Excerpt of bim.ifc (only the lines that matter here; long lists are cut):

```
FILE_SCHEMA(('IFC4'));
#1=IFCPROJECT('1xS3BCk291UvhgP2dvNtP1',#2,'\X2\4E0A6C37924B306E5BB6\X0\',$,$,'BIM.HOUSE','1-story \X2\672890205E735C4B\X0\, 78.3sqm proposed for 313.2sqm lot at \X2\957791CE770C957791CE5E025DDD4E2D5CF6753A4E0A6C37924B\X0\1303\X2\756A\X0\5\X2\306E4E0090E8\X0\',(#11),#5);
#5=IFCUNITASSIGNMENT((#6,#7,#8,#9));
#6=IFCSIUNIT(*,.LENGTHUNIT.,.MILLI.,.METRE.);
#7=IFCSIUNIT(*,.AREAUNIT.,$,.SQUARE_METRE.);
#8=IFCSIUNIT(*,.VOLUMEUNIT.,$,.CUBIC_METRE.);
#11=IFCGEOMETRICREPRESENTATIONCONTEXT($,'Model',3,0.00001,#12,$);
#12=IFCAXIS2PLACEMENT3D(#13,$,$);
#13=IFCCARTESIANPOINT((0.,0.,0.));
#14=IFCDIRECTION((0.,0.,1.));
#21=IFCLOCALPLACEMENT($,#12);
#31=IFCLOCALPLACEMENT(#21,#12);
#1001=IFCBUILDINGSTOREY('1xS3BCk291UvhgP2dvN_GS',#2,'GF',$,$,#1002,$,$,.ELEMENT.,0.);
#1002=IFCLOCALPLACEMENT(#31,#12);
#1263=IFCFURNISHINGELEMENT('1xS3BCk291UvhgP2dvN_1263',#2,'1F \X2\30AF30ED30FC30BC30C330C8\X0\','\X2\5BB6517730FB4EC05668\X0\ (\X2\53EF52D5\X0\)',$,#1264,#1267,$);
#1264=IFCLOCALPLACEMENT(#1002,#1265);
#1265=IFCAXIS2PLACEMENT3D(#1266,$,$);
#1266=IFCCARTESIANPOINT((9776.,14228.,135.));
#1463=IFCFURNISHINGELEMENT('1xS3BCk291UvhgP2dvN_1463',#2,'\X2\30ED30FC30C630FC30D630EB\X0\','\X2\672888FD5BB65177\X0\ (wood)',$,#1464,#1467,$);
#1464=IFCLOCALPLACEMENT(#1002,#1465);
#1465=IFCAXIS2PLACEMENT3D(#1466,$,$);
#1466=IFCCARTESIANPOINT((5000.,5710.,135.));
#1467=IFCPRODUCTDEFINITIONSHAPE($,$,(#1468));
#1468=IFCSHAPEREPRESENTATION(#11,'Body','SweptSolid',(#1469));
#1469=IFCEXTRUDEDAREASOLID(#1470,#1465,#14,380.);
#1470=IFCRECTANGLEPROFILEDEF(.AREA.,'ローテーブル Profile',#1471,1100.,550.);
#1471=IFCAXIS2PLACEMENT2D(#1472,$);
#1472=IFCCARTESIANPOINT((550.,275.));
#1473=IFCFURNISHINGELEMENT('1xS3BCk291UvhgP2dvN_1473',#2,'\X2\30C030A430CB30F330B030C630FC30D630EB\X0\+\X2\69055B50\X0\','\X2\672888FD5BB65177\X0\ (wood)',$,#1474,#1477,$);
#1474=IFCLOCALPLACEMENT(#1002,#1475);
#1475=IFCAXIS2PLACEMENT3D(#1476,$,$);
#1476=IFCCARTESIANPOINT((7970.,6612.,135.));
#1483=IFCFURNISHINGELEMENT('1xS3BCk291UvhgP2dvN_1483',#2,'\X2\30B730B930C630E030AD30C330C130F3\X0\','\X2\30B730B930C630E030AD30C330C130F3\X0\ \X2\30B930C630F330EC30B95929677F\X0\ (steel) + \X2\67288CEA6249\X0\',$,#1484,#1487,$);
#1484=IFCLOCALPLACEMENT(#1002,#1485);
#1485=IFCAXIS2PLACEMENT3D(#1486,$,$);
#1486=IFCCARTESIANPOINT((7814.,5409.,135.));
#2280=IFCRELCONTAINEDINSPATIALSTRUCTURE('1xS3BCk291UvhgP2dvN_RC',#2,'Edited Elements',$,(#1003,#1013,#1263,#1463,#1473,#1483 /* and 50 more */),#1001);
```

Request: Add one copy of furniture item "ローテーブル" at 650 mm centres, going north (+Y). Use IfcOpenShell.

```python
import numpy as np
import ifcopenshell
import ifcopenshell.api.geometry
import ifcopenshell.api.root
import ifcopenshell.util.element
import ifcopenshell.util.placement

model = ifcopenshell.open("bim.ifc")


def reuse_history(source, copy):
    """copy_class also copies each property set's owner history, people and application; keep the originals."""
    for rel in copy.IsDefinedBy:
        if rel.is_a("IfcRelDefinesByProperties") and (history := rel.RelatingPropertyDefinition.OwnerHistory):
            rel.RelatingPropertyDefinition.OwnerHistory = source.OwnerHistory
            ifcopenshell.util.element.remove_deep2(model, history)


source = model.by_guid("1xS3BCk291UvhgP2dvN_1463")
base = ifcopenshell.util.placement.get_local_placement(source.ObjectPlacement)
step = np.array([0.0, 1.0, 0.0]) * 650.0

for i in range(1, 2):
    copy = ifcopenshell.api.root.copy_class(model, product=source)
    copy.Representation = ifcopenshell.util.element.copy_deep(
        model, source.Representation, exclude=["IfcGeometricRepresentationContext", "IfcRepresentationMap"]
    )
    reuse_history(source, copy)
    matrix = base.copy()
    matrix[:3, 3] += i * step
    print("added at", matrix[:3, 3].round(3) + 0.0)
    ifcopenshell.api.geometry.edit_object_placement(model, product=copy, matrix=matrix, is_si=False)

model.write("bim-out.ifc")
```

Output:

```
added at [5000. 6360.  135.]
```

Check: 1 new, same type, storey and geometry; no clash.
